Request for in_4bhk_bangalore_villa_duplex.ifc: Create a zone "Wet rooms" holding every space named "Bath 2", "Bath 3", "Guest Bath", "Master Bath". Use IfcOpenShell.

First a look at what the model holds.

```python
import ifcopenshell

model = ifcopenshell.open("in_4bhk_bangalore_villa_duplex.ifc")
print(model.schema)
seen = {}
for space in model.by_type("IfcSpace"):
    seen[space.LongName] = seen.get(space.LongName, 0) + 1
for name, count in sorted(seen.items(), key=str):
    print(count, "x", name)
print("zones:", [z.Name for z in model.by_type("IfcZone")][:20])
```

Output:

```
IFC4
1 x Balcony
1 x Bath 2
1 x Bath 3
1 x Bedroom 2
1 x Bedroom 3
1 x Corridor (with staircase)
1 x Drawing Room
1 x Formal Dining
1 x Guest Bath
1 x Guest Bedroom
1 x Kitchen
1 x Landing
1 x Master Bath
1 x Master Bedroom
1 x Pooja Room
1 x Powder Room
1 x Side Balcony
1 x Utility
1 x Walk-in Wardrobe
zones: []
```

```python
import ifcopenshell
import ifcopenshell.api.group
import ifcopenshell.api.root

model = ifcopenshell.open("in_4bhk_bangalore_villa_duplex.ifc")

names = {"Bath 2", "Bath 3", "Guest Bath", "Master Bath"}
spaces = [s for s in model.by_type("IfcSpace") if s.LongName in names]

zone = ifcopenshell.api.root.create_entity(model, ifc_class="IfcZone", name="Wet rooms")
ifcopenshell.api.group.assign_group(model, products=spaces, group=zone)
print(len(spaces), "spaces in", zone.Name)

model.write("in_4bhk_bangalore_villa_duplex_rev.ifc")
```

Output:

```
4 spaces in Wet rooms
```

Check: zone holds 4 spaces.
